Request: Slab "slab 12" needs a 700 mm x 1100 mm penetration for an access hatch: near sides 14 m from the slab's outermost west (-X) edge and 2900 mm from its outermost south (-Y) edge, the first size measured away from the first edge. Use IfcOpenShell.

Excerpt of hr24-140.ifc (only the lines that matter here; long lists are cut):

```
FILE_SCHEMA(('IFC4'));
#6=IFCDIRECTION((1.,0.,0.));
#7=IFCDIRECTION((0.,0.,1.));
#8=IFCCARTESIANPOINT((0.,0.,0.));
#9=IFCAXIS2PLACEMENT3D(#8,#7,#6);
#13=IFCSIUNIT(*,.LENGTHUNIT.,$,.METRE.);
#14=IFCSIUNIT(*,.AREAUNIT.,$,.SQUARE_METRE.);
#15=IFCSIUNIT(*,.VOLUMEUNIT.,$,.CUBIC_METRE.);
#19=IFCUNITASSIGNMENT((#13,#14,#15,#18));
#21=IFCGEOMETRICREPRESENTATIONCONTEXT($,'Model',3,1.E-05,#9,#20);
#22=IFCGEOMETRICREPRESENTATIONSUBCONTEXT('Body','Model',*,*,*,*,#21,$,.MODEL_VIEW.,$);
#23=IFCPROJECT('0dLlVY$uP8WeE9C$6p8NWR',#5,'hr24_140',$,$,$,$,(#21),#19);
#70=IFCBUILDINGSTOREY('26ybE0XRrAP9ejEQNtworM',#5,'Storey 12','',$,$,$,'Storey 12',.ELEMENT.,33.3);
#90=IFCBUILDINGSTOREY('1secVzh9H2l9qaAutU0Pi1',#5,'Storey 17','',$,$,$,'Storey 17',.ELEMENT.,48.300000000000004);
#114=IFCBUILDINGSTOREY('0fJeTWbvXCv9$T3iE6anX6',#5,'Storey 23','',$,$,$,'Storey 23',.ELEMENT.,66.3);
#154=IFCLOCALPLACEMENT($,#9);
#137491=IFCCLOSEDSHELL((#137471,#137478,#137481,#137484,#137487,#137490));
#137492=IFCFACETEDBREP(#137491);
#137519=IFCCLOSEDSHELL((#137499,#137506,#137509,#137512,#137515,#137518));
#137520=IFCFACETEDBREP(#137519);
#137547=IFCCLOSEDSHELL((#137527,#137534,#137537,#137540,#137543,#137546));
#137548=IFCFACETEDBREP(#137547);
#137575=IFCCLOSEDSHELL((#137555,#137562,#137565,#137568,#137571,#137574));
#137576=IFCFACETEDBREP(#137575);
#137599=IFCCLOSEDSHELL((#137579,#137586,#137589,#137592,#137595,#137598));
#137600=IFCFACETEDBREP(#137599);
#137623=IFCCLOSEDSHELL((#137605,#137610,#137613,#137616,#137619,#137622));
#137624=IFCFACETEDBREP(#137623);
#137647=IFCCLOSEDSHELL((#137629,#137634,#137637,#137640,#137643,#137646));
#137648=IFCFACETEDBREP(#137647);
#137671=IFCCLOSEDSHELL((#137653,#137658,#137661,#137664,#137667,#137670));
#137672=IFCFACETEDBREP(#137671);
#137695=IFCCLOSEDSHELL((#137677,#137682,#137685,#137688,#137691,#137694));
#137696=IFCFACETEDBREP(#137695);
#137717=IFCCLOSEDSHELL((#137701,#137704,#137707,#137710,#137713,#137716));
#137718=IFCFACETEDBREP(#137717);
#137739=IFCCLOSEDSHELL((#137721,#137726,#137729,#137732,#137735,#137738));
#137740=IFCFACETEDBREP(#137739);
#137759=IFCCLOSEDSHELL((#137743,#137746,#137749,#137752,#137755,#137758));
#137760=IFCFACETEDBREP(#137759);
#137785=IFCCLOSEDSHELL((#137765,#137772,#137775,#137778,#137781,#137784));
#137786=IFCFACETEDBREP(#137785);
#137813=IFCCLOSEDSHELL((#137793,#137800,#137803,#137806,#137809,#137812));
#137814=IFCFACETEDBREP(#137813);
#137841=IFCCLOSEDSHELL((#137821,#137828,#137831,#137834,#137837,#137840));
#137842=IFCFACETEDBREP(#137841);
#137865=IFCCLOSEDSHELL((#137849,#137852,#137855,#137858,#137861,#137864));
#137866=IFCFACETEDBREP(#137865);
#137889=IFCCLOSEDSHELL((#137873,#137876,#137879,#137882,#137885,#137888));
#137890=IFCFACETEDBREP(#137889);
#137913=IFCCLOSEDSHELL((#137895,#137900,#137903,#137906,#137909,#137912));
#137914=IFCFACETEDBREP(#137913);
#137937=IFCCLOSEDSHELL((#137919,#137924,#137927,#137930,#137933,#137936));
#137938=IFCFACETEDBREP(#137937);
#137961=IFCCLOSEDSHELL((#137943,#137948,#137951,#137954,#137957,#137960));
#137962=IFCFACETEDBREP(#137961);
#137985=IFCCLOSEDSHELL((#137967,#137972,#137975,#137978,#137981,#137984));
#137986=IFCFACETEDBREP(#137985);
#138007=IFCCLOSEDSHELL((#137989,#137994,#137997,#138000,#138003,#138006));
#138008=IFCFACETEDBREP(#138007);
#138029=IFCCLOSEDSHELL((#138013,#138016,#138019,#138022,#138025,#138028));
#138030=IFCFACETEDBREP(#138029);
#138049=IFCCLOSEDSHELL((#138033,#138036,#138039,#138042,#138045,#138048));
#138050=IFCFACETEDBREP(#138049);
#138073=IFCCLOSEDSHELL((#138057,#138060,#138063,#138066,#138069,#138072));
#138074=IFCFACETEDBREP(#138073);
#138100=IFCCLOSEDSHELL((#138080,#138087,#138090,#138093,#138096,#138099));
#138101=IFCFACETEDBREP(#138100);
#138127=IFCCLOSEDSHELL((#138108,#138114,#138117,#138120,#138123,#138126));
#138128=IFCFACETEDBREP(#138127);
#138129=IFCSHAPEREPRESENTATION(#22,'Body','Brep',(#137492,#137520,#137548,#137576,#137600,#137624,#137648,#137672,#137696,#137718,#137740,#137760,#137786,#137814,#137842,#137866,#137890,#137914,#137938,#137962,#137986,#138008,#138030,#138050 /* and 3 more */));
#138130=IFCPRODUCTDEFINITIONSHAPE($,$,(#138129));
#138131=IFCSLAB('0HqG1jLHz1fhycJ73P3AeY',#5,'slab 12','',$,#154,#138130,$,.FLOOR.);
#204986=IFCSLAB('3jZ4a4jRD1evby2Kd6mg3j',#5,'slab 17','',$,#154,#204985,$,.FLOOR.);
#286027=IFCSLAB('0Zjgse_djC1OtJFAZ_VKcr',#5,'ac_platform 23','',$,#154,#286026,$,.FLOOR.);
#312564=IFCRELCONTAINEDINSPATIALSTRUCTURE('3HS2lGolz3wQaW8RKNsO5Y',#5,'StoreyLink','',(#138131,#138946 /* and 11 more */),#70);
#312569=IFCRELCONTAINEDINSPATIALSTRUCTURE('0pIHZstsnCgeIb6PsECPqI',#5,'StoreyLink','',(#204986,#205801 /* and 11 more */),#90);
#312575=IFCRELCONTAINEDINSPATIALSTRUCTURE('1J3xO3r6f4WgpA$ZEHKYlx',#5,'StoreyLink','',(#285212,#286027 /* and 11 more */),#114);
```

```python
import numpy as np
import ifcopenshell
import ifcopenshell.api.feature
import ifcopenshell.api.geometry
import ifcopenshell.api.root
import ifcopenshell.geom
import ifcopenshell.util.placement
import ifcopenshell.util.representation
import ifcopenshell.util.shape
import ifcopenshell.util.unit

model = ifcopenshell.open("hr24-140.ifc")
unit_scale = ifcopenshell.util.unit.calculate_unit_scale(model)
settings = ifcopenshell.geom.settings()


def volume(element):
    """Net volume in cubic metres, openings subtracted."""
    shape = ifcopenshell.geom.create_shape(settings, element)
    return ifcopenshell.util.shape.get_volume(shape.geometry)


slab = model.by_guid("0HqG1jLHz1fhycJ73P3AeY")
before = volume(slab)

# Extent in the slab's own axes, in metres. The edges named are its -X and -Y sides.
slab_shape = ifcopenshell.geom.create_shape(settings, slab)
vertices = ifcopenshell.util.shape.get_vertices(slab_shape.geometry)
x_min, y_min, bottom = vertices.min(axis=0)
top = vertices[:, 2].max()

opening = ifcopenshell.api.root.create_entity(model, ifc_class="IfcOpeningElement", name="Access hatch opening", predefined_type="OPENING")
context = ifcopenshell.util.representation.get_context(model, "Model", "Body", "MODEL_VIEW")
width, depth = 0.7, 1.1
outline = [(0.0, 0.0), (width, 0.0), (width, depth), (0.0, depth), (0.0, 0.0)]
# Overshoot both faces by 50 mm so the cut is clean.
shape = ifcopenshell.api.geometry.add_slab_representation(
    model, context=context, depth=top - bottom + 0.1, polyline=outline
)
ifcopenshell.api.geometry.assign_representation(model, product=opening, representation=shape)

matrix = ifcopenshell.util.placement.get_local_placement(slab.ObjectPlacement)
matrix[:, 3] = matrix @ np.append(np.array([x_min + 14, y_min + 2.9, bottom - 0.05]) / unit_scale, 1.0)
ifcopenshell.api.geometry.edit_object_placement(model, product=opening, matrix=matrix, is_si=False)
ifcopenshell.api.feature.add_feature(model, feature=opening, element=slab)

after = volume(slab)

print(f"slab volume {before:.3f} -> {after:.3f} m3")

model.write("hr24-140_updated.ifc")
```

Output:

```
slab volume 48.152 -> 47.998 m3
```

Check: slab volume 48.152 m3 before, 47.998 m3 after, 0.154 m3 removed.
